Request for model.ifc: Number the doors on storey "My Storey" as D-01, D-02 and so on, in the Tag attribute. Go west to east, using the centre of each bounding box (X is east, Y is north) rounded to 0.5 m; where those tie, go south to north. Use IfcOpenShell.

First a look at what the model holds.

```python
import ifcopenshell
import ifcopenshell.util.element
import ifcopenshell.util.placement

model = ifcopenshell.open("model.ifc")
print(model.schema)
storey = next(s for s in model.by_type("IfcBuildingStorey") if s.Name == "My Storey")
doors = [e for e in ifcopenshell.util.element.get_decomposition(storey) if e.is_a("IfcDoor")]
for e in sorted(doors, key=lambda e: e.id()):
    origin = ifcopenshell.util.placement.get_local_placement(e.ObjectPlacement)[:3, 3]
    print(e.id(), e.Tag, e.Name, origin.round(2) + 0.0, sep=" | ")
```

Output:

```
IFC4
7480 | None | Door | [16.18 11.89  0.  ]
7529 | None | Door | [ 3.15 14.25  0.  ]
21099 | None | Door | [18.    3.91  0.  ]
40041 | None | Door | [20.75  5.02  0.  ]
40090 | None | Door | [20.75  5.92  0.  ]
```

```python
import ifcopenshell
import ifcopenshell.geom
import ifcopenshell.util.element
import ifcopenshell.util.shape

model = ifcopenshell.open("model.ifc")
settings = ifcopenshell.geom.settings()
settings.set("use-world-coords", True)


def centre(element):
    shape = ifcopenshell.geom.create_shape(settings, element)
    return ifcopenshell.util.shape.get_bbox_centroid(shape.geometry)


storey = next(s for s in model.by_type("IfcBuildingStorey") if s.Name == "My Storey")
doors = [e for e in ifcopenshell.util.element.get_decomposition(storey) if e.is_a("IfcDoor")]

# Insertion points can sit at a corner or the storey origin, so sort by the geometry (in metres).
centres = {e: centre(e) for e in doors}
doors.sort(key=lambda e: (round(centres[e][0] / 0.5), centres[e][1]))

for i, e in enumerate(doors, start=1):
    number = f"D-{i:02d}"
    e.Tag = number
    print(e.id(), number)

model.write("model_edited.ifc")
```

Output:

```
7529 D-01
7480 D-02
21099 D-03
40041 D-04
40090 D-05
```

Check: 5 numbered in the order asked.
